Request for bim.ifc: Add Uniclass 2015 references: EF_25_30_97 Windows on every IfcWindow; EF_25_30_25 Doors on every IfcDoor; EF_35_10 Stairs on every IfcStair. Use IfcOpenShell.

First a look at what the model holds.

```python
import ifcopenshell

model = ifcopenshell.open("bim.ifc")
print(model.schema)
print("classifications:", [c.Name for c in model.by_type("IfcClassification")])
for ifc_class in ("IfcDoor", "IfcRoof", "IfcStair", "IfcWall", "IfcWindow"):
    print(ifc_class, len(model.by_type(ifc_class)))
```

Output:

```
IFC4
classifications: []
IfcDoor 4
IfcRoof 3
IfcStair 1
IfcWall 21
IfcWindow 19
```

```python
import ifcopenshell
import ifcopenshell.api.classification

model = ifcopenshell.open("bim.ifc")

system = ifcopenshell.api.classification.add_classification(model, classification="Uniclass 2015")

codes = {
    "IfcWindow": ("EF_25_30_97", "Windows"),
    "IfcDoor": ("EF_25_30_25", "Doors"),
    "IfcStair": ("EF_35_10", "Stairs"),
}
for ifc_class, (code, name) in codes.items():
    products = model.by_type(ifc_class)
    ifcopenshell.api.classification.add_reference(
        model, products=products, classification=system, identification=code, name=name
    )
    print(code, len(products))

model.write("bim_edited.ifc")
```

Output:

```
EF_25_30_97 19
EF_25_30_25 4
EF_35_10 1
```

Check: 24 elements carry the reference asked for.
